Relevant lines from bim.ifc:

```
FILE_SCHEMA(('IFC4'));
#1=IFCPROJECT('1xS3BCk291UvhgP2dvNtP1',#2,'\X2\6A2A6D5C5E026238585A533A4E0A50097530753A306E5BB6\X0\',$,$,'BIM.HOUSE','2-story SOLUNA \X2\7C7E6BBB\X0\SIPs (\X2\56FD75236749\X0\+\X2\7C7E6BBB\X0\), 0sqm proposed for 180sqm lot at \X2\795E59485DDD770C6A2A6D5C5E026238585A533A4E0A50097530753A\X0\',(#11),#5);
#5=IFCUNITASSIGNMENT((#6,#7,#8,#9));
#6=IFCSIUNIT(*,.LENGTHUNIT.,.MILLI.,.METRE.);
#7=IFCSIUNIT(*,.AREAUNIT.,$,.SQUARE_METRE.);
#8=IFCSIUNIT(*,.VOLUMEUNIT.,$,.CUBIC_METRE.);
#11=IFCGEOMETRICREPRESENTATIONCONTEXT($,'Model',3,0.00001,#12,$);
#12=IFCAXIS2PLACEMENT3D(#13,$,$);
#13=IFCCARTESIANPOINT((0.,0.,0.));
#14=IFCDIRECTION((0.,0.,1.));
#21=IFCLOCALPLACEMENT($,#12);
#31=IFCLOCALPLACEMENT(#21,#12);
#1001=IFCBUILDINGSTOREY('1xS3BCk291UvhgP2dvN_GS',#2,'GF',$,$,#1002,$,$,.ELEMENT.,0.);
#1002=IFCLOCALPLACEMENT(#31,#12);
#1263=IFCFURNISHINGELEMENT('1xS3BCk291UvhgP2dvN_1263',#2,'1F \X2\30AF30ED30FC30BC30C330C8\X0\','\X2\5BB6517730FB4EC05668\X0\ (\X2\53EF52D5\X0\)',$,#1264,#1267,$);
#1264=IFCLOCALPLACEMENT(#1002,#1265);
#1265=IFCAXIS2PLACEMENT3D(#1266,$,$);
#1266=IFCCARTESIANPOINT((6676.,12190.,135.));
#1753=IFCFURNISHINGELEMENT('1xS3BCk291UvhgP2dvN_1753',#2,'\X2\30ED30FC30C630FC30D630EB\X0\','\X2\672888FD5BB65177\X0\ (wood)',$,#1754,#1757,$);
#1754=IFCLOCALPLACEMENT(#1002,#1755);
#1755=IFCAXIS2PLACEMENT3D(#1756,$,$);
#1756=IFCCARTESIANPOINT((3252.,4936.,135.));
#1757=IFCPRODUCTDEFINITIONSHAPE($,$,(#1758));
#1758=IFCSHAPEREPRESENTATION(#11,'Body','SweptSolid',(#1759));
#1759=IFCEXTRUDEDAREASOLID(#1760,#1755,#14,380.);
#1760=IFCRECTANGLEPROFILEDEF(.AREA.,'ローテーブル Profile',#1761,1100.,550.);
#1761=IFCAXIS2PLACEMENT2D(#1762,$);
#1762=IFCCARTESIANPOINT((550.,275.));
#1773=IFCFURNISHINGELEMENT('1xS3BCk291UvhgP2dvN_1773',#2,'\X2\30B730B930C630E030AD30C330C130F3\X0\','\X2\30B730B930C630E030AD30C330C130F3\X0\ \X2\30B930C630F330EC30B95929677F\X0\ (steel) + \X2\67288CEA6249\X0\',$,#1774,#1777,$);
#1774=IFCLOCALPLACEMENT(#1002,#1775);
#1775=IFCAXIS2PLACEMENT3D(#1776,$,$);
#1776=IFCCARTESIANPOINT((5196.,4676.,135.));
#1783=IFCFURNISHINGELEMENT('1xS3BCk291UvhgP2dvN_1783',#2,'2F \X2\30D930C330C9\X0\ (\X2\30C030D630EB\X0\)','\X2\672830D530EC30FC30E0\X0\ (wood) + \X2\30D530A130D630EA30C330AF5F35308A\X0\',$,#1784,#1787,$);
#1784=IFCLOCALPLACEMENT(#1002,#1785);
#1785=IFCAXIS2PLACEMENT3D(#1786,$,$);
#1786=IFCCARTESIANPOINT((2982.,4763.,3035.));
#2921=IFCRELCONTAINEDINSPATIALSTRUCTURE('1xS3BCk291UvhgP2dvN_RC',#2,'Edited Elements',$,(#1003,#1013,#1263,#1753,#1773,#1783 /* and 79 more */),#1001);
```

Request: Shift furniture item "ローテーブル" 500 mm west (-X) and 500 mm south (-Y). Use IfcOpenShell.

```python
import ifcopenshell
import ifcopenshell.api.geometry
import ifcopenshell.util.placement

model = ifcopenshell.open("bim.ifc")

item = model.by_guid("1xS3BCk291UvhgP2dvN_1753")
matrix = ifcopenshell.util.placement.get_local_placement(item.ObjectPlacement)
matrix[0, 3] -= 500.0
matrix[1, 3] -= 500.0
ifcopenshell.api.geometry.edit_object_placement(model, product=item, matrix=matrix, is_si=False)

print(ifcopenshell.util.placement.get_local_placement(item.ObjectPlacement).round(3) + 0.0)

model.write("bim_updated.ifc")
```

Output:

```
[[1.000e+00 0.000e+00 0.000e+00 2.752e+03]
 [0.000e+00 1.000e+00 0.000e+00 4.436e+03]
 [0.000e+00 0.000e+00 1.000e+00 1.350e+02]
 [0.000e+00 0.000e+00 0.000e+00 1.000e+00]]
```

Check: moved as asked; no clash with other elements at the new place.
